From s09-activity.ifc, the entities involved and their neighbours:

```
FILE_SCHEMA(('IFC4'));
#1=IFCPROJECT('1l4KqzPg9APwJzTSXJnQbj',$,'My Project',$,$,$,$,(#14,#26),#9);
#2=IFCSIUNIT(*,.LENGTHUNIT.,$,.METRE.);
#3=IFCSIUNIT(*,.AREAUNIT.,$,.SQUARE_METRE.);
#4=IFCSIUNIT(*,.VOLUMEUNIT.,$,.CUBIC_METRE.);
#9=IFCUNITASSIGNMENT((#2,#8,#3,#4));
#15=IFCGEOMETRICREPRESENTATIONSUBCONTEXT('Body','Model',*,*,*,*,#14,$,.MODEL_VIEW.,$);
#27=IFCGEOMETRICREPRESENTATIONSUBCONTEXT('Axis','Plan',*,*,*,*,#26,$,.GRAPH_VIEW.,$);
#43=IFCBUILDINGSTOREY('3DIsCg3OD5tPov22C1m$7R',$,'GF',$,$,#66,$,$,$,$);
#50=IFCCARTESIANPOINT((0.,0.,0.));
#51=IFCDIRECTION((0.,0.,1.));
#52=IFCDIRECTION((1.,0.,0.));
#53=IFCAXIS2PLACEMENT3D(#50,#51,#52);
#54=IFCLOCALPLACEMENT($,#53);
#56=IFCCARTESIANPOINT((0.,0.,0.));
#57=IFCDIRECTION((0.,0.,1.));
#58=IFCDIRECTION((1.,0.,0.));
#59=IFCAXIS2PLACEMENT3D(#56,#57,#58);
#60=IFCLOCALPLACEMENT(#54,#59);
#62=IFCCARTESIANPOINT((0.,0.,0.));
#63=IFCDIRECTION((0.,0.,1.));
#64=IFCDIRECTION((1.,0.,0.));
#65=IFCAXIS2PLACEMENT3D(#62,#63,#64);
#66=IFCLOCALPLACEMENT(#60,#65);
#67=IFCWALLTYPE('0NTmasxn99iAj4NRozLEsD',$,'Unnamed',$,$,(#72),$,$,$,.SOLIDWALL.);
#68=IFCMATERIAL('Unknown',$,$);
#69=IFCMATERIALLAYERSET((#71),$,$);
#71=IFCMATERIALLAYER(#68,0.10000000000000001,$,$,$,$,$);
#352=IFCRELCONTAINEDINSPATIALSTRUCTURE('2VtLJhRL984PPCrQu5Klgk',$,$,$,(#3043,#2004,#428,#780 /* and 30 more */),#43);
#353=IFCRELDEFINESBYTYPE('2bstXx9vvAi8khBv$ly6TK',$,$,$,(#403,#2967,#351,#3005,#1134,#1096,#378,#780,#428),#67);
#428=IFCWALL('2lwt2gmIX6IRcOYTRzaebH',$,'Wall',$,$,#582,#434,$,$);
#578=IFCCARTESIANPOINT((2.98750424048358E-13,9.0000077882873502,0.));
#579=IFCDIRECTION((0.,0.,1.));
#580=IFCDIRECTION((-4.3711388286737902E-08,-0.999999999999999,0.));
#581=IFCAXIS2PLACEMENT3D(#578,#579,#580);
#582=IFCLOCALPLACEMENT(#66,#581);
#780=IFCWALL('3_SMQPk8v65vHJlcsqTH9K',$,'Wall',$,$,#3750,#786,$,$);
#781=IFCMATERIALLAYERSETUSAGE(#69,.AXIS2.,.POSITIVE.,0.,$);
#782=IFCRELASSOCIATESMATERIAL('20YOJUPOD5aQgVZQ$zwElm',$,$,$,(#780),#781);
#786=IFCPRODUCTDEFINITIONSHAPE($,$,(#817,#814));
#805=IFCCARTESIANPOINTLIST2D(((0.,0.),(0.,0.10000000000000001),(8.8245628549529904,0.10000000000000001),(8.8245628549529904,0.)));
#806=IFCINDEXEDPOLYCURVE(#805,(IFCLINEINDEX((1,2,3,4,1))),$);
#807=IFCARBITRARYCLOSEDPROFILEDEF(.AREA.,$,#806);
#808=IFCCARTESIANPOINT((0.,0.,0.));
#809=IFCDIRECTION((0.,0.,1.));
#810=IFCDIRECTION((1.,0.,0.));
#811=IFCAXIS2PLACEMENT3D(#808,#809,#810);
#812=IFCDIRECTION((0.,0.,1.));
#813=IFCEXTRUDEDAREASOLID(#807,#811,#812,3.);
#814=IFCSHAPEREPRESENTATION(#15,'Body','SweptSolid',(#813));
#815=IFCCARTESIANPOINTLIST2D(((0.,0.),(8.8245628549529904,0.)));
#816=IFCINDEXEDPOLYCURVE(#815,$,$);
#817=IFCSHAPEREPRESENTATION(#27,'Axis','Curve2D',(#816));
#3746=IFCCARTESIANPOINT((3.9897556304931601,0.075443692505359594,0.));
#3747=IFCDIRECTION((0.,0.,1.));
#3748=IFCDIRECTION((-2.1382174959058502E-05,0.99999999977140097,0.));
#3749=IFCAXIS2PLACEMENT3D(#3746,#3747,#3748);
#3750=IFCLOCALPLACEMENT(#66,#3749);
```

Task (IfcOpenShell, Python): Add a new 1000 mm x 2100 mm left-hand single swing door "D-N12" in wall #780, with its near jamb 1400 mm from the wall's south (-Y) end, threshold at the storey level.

```python
import numpy as np
import ifcopenshell
import ifcopenshell.api.feature
import ifcopenshell.api.geometry
import ifcopenshell.api.root
import ifcopenshell.api.spatial
import ifcopenshell.geom
import ifcopenshell.util.element
import ifcopenshell.util.placement
import ifcopenshell.util.representation
import ifcopenshell.util.shape
import ifcopenshell.util.unit

model = ifcopenshell.open("s09-activity.ifc")
unit_scale = ifcopenshell.util.unit.calculate_unit_scale(model)
settings = ifcopenshell.geom.settings()


def volume(element):
    """Net volume in cubic metres, openings subtracted."""
    shape = ifcopenshell.geom.create_shape(settings, element)
    return ifcopenshell.util.shape.get_volume(shape.geometry)


wall = model.by_id(780)
storey = ifcopenshell.util.element.get_container(wall, ifc_class="IfcBuildingStorey")
context = ifcopenshell.util.representation.get_context(model, "Model", "Body", "MODEL_VIEW")
before = volume(wall)

width, height, from_end, sill = 1, 2.1, 1.4, 0.0  # metres

# The wall runs along its own X axis, and the end named is its -X end.
wall_shape = ifcopenshell.geom.create_shape(settings, wall)
x, y, z = ifcopenshell.util.shape.get_vertices(wall_shape.geometry).T
start = x.min() + from_end
face, thickness = float(y.min()), float(y.max() - y.min())
wall_matrix = ifcopenshell.util.placement.get_local_placement(wall.ObjectPlacement)
level = ifcopenshell.util.placement.get_local_placement(storey.ObjectPlacement)[2, 3]


def in_wall(x, y):
    """Placement at x, y metres in the wall's axes, at sill height."""
    matrix = wall_matrix.copy()
    matrix[:, 3] = wall_matrix @ np.array([x / unit_scale, y / unit_scale, 0.0, 1.0])
    matrix[2, 3] = level + sill / unit_scale
    return matrix


# Opening: a box that overshoots both wall faces by 50 mm.
opening = ifcopenshell.api.root.create_entity(model, ifc_class="IfcOpeningElement", predefined_type="OPENING")
box = ifcopenshell.api.geometry.add_wall_representation(
    model, context=context, length=width, height=height, thickness=thickness + 0.1
)
ifcopenshell.api.geometry.assign_representation(model, product=opening, representation=box)
ifcopenshell.api.geometry.edit_object_placement(model, product=opening, matrix=in_wall(start, face - 0.05), is_si=False)
ifcopenshell.api.feature.add_feature(model, feature=opening, element=wall)

door = ifcopenshell.api.root.create_entity(model, ifc_class="IfcDoor", name="D-N12", predefined_type="DOOR")
door.OverallWidth, door.OverallHeight = width / unit_scale, height / unit_scale
door.OperationType = "SINGLE_SWING_LEFT"
body = ifcopenshell.api.geometry.add_door_representation(
    model,
    context=context,
    overall_width=door.OverallWidth,
    overall_height=door.OverallHeight,
    operation_type="SINGLE_SWING_LEFT",
    lining_properties={"LiningDepth": thickness / unit_scale, "ThresholdDepth": thickness / unit_scale},
)
ifcopenshell.api.geometry.assign_representation(model, product=door, representation=body)
ifcopenshell.api.spatial.assign_container(model, products=[door], relating_structure=storey)
ifcopenshell.api.feature.add_filling(model, opening=opening, element=door)

# The lining spans the wall, so the door starts at the wall face.
ifcopenshell.api.geometry.edit_object_placement(model, product=door, matrix=in_wall(start, face), is_si=False)

after = volume(wall)

print(f"wall volume {before:.3f} -> {after:.3f} m3")

model.write("s09-activity_updated.ifc")
```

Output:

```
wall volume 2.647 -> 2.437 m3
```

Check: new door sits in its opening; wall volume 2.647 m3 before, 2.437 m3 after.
